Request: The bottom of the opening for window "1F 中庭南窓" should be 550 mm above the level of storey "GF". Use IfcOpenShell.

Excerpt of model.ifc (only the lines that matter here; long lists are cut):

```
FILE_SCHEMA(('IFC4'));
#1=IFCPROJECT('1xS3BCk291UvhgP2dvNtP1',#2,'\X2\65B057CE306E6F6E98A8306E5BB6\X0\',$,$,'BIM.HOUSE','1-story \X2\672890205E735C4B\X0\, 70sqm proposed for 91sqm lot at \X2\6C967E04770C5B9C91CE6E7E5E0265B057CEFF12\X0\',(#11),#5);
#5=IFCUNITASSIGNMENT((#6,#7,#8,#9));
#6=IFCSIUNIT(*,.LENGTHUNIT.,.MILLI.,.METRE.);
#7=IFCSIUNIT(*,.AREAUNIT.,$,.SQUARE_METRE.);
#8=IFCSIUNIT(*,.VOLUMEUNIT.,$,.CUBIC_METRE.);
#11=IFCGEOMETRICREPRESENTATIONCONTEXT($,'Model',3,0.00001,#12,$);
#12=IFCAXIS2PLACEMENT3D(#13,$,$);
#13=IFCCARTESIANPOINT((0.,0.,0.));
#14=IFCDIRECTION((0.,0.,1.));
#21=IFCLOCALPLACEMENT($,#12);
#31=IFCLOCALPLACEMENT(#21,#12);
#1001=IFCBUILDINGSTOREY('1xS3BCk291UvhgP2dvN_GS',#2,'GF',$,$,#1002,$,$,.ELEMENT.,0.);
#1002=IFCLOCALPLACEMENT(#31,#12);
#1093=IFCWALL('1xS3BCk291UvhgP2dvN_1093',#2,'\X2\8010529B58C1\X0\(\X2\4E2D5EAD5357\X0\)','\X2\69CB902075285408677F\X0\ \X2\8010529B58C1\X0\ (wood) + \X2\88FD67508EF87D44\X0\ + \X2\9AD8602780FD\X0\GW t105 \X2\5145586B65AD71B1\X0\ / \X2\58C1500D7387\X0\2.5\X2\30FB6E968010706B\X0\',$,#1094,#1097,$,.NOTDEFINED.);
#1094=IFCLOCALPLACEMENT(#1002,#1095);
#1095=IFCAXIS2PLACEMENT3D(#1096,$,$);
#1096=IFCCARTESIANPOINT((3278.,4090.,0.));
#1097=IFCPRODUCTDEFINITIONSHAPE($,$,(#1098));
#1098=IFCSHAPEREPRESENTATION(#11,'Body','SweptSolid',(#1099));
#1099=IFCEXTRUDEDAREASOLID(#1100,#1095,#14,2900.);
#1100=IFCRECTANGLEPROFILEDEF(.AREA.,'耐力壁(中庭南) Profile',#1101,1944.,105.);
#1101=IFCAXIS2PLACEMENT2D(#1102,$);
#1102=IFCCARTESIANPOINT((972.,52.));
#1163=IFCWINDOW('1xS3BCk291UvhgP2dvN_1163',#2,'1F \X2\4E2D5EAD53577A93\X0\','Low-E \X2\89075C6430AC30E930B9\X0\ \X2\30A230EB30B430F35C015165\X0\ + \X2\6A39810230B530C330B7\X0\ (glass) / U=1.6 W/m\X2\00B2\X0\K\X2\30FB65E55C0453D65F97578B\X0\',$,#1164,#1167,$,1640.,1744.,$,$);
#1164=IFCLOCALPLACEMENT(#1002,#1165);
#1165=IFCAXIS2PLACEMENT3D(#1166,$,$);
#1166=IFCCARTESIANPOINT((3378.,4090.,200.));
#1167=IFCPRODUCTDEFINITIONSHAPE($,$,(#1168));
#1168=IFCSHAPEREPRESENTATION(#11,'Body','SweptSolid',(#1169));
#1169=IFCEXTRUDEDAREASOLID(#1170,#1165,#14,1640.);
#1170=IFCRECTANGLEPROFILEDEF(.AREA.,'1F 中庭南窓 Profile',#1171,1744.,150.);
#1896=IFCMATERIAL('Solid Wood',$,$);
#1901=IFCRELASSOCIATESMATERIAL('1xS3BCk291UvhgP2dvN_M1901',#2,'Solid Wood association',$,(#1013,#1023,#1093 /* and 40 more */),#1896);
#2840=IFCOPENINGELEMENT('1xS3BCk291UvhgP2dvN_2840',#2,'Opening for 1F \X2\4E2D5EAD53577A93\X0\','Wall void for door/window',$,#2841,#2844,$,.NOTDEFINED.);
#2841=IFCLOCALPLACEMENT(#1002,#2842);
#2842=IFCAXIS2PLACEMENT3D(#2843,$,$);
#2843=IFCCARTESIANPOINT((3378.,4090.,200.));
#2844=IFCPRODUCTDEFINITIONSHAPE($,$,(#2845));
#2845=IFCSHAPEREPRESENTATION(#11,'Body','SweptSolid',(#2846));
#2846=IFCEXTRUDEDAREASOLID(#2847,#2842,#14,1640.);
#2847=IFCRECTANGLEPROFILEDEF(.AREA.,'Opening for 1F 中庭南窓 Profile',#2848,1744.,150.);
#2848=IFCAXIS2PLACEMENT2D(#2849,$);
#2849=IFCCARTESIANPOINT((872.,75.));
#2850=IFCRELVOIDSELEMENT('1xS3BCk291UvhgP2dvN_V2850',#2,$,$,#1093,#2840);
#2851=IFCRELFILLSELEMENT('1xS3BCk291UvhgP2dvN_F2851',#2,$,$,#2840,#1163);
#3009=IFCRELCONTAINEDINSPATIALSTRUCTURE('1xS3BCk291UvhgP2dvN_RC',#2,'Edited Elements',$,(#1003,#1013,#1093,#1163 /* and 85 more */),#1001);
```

```python
import numpy as np
import ifcopenshell
import ifcopenshell.api.geometry
import ifcopenshell.geom
import ifcopenshell.util.element
import ifcopenshell.util.placement
import ifcopenshell.util.shape
import ifcopenshell.util.unit

model = ifcopenshell.open("model.ifc")
unit_scale = ifcopenshell.util.unit.calculate_unit_scale(model)

window = model.by_id(1163)
opening = window.FillsVoids[0].RelatingOpeningElement
storey = ifcopenshell.util.element.get_container(window, ifc_class="IfcBuildingStorey")
level = ifcopenshell.util.placement.get_local_placement(storey.ObjectPlacement)[2, 3]

# The opening's origin need not be at the sill, so measure its lowest point.
shape = ifcopenshell.geom.create_shape(ifcopenshell.geom.settings(), opening)
bottom = ifcopenshell.util.shape.get_shape_bottom_elevation(shape, shape.geometry) / unit_scale
dz = level + 550.0 - bottom

shift = np.array([0.0, 0.0, dz])
# The window is not placed relative to its opening, so move both.
for product in (opening, window):
    matrix = ifcopenshell.util.placement.get_local_placement(product.ObjectPlacement)
    matrix[:3, 3] += shift
    ifcopenshell.api.geometry.edit_object_placement(model, product=product, matrix=matrix, is_si=False)

print(f"moved by {dz * unit_scale:+.3f} m")

model.write("model_v2.ifc")
```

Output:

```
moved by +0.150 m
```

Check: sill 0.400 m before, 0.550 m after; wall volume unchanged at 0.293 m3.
